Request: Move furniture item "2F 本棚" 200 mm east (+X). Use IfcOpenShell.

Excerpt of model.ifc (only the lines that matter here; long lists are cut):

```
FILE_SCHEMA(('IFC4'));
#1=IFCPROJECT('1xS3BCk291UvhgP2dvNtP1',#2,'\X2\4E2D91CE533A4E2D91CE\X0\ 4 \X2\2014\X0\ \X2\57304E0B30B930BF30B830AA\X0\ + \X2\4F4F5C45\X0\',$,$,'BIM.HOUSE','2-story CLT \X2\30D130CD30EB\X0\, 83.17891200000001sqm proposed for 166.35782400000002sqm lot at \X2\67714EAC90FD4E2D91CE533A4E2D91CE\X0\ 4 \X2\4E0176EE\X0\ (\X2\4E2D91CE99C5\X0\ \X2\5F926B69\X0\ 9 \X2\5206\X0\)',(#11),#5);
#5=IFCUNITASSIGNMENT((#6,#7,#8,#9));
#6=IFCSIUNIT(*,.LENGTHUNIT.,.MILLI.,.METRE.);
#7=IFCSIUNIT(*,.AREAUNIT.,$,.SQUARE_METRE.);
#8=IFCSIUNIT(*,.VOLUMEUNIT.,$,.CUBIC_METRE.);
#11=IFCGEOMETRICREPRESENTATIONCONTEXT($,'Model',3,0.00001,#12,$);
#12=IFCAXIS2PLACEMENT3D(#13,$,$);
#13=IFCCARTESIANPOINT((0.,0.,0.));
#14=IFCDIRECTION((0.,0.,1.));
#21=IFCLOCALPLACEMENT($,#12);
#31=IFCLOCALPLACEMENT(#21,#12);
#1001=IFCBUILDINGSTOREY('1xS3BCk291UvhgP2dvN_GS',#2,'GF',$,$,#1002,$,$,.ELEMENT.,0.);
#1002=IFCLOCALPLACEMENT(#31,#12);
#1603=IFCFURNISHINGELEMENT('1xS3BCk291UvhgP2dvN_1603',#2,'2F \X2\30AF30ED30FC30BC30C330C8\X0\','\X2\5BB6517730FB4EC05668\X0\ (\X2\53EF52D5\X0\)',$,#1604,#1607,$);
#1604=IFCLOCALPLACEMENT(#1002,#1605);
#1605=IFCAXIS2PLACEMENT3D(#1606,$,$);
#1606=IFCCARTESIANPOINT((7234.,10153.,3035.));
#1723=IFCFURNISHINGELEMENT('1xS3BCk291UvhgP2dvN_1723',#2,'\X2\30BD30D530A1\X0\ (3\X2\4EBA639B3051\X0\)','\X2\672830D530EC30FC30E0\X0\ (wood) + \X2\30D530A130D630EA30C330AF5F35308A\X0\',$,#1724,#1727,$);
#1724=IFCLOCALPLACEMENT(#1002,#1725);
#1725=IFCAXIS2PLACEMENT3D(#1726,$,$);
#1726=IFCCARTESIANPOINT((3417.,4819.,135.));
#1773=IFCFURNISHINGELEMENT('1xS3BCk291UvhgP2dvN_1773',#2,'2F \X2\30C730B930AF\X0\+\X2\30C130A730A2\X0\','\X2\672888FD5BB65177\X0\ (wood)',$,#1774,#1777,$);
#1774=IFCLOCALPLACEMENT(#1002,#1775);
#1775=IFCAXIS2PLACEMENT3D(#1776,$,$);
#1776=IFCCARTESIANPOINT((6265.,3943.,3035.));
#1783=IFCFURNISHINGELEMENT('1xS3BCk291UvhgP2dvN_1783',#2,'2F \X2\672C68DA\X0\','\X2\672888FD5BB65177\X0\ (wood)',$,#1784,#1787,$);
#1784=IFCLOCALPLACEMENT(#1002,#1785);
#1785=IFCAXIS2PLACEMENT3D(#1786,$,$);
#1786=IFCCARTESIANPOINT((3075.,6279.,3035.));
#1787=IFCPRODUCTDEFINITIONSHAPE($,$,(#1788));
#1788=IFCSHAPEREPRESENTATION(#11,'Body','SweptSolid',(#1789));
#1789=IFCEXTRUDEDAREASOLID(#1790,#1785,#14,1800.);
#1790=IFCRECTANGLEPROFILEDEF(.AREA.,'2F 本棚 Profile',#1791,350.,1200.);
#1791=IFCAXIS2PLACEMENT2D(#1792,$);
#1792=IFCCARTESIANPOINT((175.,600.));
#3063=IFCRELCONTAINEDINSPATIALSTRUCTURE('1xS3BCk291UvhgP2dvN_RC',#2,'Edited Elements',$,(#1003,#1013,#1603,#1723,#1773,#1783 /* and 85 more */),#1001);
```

```python
import ifcopenshell
import ifcopenshell.api.geometry
import ifcopenshell.util.placement
import ifcopenshell.util.unit

model = ifcopenshell.open("model.ifc")
unit_scale = ifcopenshell.util.unit.calculate_unit_scale(model)

item = model.by_guid("1xS3BCk291UvhgP2dvN_1783")
matrix = ifcopenshell.util.placement.get_local_placement(item.ObjectPlacement)
matrix[0, 3] += 0.2 / unit_scale
ifcopenshell.api.geometry.edit_object_placement(model, product=item, matrix=matrix, is_si=False)

print(ifcopenshell.util.placement.get_local_placement(item.ObjectPlacement).round(3) + 0.0)

model.write("model_edited.ifc")
```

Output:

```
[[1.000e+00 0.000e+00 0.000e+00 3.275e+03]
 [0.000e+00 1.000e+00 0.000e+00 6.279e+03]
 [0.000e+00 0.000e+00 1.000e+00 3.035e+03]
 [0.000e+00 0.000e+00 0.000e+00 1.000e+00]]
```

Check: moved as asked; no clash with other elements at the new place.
